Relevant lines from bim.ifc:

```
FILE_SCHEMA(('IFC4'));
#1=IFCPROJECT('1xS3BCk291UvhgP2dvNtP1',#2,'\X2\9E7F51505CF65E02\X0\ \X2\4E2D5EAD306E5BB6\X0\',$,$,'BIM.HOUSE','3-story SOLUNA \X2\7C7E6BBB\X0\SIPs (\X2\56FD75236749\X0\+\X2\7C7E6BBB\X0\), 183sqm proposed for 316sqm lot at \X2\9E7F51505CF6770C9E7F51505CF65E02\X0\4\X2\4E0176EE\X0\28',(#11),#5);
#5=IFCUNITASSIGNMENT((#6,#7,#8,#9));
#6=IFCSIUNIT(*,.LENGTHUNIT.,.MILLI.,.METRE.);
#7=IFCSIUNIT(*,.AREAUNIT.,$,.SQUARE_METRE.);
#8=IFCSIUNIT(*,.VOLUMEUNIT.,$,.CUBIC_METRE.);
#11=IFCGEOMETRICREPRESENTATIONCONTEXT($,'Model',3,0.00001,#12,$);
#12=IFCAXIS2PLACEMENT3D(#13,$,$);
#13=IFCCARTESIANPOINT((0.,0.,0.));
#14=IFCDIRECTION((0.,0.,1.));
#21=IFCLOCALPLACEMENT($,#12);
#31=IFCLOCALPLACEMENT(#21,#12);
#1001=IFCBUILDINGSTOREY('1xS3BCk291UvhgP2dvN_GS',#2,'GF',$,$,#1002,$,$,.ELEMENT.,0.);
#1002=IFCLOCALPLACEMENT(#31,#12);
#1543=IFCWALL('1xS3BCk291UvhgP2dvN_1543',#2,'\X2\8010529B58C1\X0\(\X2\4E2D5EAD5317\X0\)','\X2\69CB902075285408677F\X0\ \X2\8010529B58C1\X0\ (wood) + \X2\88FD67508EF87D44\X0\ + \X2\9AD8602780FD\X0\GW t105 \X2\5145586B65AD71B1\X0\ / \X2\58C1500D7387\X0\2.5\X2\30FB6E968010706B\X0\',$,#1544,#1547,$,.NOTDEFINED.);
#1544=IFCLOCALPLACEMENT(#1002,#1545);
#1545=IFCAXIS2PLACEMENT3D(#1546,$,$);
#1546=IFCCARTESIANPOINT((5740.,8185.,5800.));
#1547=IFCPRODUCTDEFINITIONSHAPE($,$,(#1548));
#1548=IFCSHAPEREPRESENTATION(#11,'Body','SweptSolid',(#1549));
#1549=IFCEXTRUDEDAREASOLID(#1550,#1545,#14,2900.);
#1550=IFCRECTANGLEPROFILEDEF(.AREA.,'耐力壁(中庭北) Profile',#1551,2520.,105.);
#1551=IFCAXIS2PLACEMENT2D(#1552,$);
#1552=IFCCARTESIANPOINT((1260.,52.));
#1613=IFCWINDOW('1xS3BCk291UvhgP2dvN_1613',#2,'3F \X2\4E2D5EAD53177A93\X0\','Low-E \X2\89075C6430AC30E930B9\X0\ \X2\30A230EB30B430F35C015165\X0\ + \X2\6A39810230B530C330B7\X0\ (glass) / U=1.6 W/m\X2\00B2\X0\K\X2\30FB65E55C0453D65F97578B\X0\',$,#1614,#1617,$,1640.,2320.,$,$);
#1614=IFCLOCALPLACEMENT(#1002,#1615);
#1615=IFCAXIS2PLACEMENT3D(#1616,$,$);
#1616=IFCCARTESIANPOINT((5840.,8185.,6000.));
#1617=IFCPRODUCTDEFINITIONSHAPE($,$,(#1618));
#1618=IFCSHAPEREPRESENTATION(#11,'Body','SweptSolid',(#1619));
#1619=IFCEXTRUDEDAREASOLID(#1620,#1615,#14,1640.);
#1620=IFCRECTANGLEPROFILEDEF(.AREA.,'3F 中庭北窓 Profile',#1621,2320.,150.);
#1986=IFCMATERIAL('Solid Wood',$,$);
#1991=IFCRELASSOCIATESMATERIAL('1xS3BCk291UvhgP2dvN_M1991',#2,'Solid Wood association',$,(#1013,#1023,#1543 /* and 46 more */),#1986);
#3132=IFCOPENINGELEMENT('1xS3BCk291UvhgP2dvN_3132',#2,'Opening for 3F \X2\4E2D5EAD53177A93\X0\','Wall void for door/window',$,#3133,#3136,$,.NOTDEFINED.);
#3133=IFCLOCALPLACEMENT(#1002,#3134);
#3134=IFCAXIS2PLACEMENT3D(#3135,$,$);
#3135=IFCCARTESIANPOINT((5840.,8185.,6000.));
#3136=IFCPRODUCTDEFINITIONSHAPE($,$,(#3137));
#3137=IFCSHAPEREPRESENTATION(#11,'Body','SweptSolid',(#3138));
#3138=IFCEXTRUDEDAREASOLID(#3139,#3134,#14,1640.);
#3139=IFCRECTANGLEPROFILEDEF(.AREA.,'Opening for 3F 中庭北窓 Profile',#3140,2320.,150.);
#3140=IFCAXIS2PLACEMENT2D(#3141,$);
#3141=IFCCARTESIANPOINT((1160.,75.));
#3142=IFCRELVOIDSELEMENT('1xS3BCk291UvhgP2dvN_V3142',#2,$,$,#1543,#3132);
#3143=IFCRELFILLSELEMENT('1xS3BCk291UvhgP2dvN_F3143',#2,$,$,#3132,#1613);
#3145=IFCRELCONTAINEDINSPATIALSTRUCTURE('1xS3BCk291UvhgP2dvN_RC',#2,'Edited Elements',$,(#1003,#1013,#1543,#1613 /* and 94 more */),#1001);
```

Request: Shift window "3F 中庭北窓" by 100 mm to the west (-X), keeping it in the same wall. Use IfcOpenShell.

```python
import ifcopenshell
import ifcopenshell.api.geometry
import ifcopenshell.util.placement
import ifcopenshell.util.unit

model = ifcopenshell.open("bim.ifc")
unit_scale = ifcopenshell.util.unit.calculate_unit_scale(model)

window = model.by_guid("1xS3BCk291UvhgP2dvN_1613")
opening = window.FillsVoids[0].RelatingOpeningElement
wall = opening.VoidsElements[0].RelatingBuildingElement

wall_matrix = ifcopenshell.util.placement.get_local_placement(wall.ObjectPlacement)
shift = wall_matrix[:3, 0] * -0.1 / unit_scale
before = ifcopenshell.util.placement.get_local_placement(window.ObjectPlacement)[:3, 3].copy()

# The window is not placed relative to its opening, so move both.
for product in (opening, window):
    matrix = ifcopenshell.util.placement.get_local_placement(product.ObjectPlacement)
    matrix[:3, 3] += shift
    ifcopenshell.api.geometry.edit_object_placement(model, product=product, matrix=matrix, is_si=False)

after = ifcopenshell.util.placement.get_local_placement(window.ObjectPlacement)[:3, 3]
print("window moved by", (after - before).round(3) + 0.0)

model.write("bim_edited.ifc")
```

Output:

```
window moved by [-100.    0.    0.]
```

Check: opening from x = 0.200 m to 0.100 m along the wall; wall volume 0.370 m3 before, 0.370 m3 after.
